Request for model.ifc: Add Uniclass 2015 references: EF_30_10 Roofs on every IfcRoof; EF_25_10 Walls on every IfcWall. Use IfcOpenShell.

First a look at what the model holds.

```python
import ifcopenshell

model = ifcopenshell.open("model.ifc")
print(model.schema)
print("classifications:", [c.Name for c in model.by_type("IfcClassification")])
for ifc_class in ("IfcDoor", "IfcRoof", "IfcStair", "IfcWall", "IfcWindow"):
    print(ifc_class, len(model.by_type(ifc_class)))
```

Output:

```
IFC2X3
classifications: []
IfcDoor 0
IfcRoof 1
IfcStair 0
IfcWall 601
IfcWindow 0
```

```python
import ifcopenshell
import ifcopenshell.api.classification

model = ifcopenshell.open("model.ifc")

# IFC2X3 requires Source and Edition and has no link from the project to the system.
system = model.create_entity("IfcClassification", Source="NBS", Edition="2015", Name="Uniclass 2015")

codes = {
    "IfcRoof": ("EF_30_10", "Roofs"),
    "IfcWall": ("EF_25_10", "Walls"),
}
for ifc_class, (code, name) in codes.items():
    products = model.by_type(ifc_class)
    ifcopenshell.api.classification.add_reference(
        model, products=products, classification=system, identification=code, name=name
    )
    print(code, len(products))

model.write("model_rev.ifc")
```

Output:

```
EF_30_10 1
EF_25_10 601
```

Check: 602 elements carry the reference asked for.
